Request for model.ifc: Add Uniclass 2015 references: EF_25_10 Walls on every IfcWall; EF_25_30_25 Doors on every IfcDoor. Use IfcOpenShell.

First a look at what the model holds.

```python
import ifcopenshell

model = ifcopenshell.open("model.ifc")
print(model.schema)
print("classifications:", [c.Name for c in model.by_type("IfcClassification")])
for ifc_class in ("IfcDoor", "IfcRoof", "IfcStair", "IfcWall", "IfcWindow"):
    print(ifc_class, len(model.by_type(ifc_class)))
```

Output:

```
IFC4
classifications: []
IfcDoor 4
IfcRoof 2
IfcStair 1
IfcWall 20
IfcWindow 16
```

```python
import ifcopenshell
import ifcopenshell.api.classification

model = ifcopenshell.open("model.ifc")

system = ifcopenshell.api.classification.add_classification(model, classification="Uniclass 2015")

codes = {
    "IfcWall": ("EF_25_10", "Walls"),
    "IfcDoor": ("EF_25_30_25", "Doors"),
}
for ifc_class, (code, name) in codes.items():
    products = model.by_type(ifc_class)
    ifcopenshell.api.classification.add_reference(
        model, products=products, classification=system, identification=code, name=name
    )
    print(code, len(products))

model.write("model_edited.ifc")
```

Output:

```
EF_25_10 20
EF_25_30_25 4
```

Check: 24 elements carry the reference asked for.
